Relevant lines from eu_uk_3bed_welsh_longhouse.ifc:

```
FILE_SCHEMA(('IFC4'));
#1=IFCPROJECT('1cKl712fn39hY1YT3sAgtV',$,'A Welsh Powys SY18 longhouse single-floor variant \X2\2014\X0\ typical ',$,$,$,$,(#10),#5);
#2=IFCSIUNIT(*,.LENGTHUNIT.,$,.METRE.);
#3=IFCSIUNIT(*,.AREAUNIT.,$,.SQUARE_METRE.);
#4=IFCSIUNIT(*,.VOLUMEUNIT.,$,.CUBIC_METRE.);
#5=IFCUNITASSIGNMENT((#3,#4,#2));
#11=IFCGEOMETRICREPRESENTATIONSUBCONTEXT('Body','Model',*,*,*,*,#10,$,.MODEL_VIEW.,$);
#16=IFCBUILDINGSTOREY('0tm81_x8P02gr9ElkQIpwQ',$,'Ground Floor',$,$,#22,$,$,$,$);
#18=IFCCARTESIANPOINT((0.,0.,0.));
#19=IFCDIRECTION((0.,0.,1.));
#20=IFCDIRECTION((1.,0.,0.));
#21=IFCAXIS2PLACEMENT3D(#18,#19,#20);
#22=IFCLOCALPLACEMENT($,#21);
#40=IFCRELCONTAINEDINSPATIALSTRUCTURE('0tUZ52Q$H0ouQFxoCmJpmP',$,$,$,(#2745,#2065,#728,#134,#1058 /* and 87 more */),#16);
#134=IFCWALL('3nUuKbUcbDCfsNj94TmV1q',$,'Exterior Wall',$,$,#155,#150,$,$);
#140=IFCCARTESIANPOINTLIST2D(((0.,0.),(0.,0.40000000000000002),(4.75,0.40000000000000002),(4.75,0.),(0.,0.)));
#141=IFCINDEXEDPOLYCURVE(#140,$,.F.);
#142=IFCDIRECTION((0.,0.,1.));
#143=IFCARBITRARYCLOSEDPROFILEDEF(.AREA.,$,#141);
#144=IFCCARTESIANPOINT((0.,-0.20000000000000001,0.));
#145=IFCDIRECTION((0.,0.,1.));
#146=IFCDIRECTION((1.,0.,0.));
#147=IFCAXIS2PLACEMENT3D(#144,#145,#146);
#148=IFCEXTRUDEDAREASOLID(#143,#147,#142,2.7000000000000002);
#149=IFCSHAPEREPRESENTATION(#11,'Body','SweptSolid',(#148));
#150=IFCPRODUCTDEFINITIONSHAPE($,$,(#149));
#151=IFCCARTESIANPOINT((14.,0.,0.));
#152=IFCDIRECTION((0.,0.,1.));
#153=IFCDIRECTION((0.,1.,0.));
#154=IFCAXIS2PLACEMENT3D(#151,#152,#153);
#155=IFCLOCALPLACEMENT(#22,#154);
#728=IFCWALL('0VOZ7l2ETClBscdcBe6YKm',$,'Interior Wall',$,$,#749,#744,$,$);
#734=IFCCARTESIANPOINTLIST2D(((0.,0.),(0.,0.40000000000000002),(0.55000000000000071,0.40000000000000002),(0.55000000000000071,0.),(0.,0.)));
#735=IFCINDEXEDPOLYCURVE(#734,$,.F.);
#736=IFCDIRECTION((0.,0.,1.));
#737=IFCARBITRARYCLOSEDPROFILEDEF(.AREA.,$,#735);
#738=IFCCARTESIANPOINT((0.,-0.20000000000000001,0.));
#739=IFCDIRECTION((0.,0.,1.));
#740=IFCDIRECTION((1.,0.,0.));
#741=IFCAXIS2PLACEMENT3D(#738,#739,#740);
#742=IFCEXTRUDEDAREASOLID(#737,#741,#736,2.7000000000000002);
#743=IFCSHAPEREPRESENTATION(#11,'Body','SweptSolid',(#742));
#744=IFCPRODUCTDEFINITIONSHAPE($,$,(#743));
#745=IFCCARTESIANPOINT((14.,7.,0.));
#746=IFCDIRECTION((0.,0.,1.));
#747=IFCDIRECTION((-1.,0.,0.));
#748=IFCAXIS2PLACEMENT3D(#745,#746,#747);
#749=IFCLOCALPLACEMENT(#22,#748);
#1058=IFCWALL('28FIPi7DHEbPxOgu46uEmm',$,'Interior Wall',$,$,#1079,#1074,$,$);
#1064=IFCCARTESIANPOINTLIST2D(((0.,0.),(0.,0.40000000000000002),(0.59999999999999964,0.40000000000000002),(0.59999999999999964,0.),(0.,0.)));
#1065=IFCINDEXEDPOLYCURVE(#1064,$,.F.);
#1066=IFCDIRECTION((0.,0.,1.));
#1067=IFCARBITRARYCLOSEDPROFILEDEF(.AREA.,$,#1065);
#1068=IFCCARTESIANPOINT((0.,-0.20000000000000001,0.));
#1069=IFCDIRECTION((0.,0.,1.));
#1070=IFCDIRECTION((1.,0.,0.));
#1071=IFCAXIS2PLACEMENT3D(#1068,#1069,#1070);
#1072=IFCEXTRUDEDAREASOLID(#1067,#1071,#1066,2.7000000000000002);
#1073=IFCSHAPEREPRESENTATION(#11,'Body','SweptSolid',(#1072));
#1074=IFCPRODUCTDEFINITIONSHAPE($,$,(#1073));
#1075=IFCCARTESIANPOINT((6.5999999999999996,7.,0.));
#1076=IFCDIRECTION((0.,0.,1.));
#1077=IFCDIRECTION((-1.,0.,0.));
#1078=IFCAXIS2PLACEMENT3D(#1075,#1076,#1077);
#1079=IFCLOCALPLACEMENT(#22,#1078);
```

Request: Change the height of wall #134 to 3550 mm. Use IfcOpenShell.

```python
import ifcopenshell
import ifcopenshell.geom
import ifcopenshell.util.representation
import ifcopenshell.util.shape

model = ifcopenshell.open("eu_uk_3bed_welsh_longhouse.ifc")
settings = ifcopenshell.geom.settings()


def volume(element):
    """Net volume in cubic metres, openings subtracted."""
    shape = ifcopenshell.geom.create_shape(settings, element)
    return ifcopenshell.util.shape.get_volume(shape.geometry)


wall = model.by_guid("3nUuKbUcbDCfsNj94TmV1q")
before = volume(wall)

body = ifcopenshell.util.representation.get_representation(wall, "Model", "Body")
solid = body.Items[0]
old_height = solid.Depth
solid.Depth = 3.55
after = volume(wall)

print(f"height {old_height:g} -> {solid.Depth:g}, volume {before:.3f} -> {after:.3f} m3")

model.write("eu_uk_3bed_welsh_longhouse_v2.ifc")
```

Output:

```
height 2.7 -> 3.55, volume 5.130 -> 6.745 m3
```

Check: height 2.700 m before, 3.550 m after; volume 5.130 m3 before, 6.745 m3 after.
